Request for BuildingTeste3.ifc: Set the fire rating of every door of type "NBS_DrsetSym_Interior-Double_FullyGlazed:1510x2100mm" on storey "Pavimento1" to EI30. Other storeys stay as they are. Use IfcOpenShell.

First a look at what the model holds.

```python
import ifcopenshell
import ifcopenshell.util.element

model = ifcopenshell.open("BuildingTeste3.ifc")
print(model.schema)
storey = next(s for s in model.by_type("IfcBuildingStorey") if s.Name == "Pavimento1")
doors = [e for e in ifcopenshell.util.element.get_decomposition(storey) if e.is_a("IfcDoor")]
seen = {}
for e in doors:
    element_type = ifcopenshell.util.element.get_type(e)
    key = (element_type.Name if element_type != e and element_type else None, ifcopenshell.util.element.get_pset(e, "Pset_DoorCommon", "FireRating"))
    seen[key] = seen.get(key, 0) + 1
for (name, value), count in sorted(seen.items(), key=str):
    print(count, "x", name, "|", value)
```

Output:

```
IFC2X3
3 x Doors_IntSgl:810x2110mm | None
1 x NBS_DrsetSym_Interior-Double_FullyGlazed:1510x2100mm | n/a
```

```python
import ifcopenshell
import ifcopenshell.api.pset
import ifcopenshell.util.element

model = ifcopenshell.open("BuildingTeste3.ifc")

storey = next(s for s in model.by_type("IfcBuildingStorey") if s.Name == "Pavimento1")
doors = [e for e in ifcopenshell.util.element.get_decomposition(storey) if e.is_a("IfcDoor")]

count = 0
for e in doors:
    element_type = ifcopenshell.util.element.get_type(e)
    if element_type in (None, e) or element_type.Name != "NBS_DrsetSym_Interior-Double_FullyGlazed:1510x2100mm":
        continue
    # add_pset returns the element's existing set when there is one.
    pset = ifcopenshell.api.pset.add_pset(model, product=e, name="Pset_DoorCommon")
    ifcopenshell.api.pset.edit_pset(model, pset=pset, properties={"FireRating": "EI30"})
    count += 1

print(count, "doors updated")

model.write("BuildingTeste3_v2.ifc")
```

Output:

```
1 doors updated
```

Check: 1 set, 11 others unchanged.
